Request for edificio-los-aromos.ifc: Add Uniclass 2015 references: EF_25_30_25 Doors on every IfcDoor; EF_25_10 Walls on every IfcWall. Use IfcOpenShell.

First a look at what the model holds.

```python
import ifcopenshell

model = ifcopenshell.open("edificio-los-aromos.ifc")
print(model.schema)
print("classifications:", [c.Name for c in model.by_type("IfcClassification")])
for ifc_class in ("IfcDoor", "IfcRoof", "IfcStair", "IfcWall", "IfcWindow"):
    print(ifc_class, len(model.by_type(ifc_class)))
```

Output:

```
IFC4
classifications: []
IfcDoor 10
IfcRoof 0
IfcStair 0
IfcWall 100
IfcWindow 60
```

```python
import ifcopenshell
import ifcopenshell.api.classification

model = ifcopenshell.open("edificio-los-aromos.ifc")

system = ifcopenshell.api.classification.add_classification(model, classification="Uniclass 2015")

codes = {
    "IfcDoor": ("EF_25_30_25", "Doors"),
    "IfcWall": ("EF_25_10", "Walls"),
}
for ifc_class, (code, name) in codes.items():
    products = model.by_type(ifc_class)
    ifcopenshell.api.classification.add_reference(
        model, products=products, classification=system, identification=code, name=name
    )
    print(code, len(products))

model.write("edificio-los-aromos_updated.ifc")
```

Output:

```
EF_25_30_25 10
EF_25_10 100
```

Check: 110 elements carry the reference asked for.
